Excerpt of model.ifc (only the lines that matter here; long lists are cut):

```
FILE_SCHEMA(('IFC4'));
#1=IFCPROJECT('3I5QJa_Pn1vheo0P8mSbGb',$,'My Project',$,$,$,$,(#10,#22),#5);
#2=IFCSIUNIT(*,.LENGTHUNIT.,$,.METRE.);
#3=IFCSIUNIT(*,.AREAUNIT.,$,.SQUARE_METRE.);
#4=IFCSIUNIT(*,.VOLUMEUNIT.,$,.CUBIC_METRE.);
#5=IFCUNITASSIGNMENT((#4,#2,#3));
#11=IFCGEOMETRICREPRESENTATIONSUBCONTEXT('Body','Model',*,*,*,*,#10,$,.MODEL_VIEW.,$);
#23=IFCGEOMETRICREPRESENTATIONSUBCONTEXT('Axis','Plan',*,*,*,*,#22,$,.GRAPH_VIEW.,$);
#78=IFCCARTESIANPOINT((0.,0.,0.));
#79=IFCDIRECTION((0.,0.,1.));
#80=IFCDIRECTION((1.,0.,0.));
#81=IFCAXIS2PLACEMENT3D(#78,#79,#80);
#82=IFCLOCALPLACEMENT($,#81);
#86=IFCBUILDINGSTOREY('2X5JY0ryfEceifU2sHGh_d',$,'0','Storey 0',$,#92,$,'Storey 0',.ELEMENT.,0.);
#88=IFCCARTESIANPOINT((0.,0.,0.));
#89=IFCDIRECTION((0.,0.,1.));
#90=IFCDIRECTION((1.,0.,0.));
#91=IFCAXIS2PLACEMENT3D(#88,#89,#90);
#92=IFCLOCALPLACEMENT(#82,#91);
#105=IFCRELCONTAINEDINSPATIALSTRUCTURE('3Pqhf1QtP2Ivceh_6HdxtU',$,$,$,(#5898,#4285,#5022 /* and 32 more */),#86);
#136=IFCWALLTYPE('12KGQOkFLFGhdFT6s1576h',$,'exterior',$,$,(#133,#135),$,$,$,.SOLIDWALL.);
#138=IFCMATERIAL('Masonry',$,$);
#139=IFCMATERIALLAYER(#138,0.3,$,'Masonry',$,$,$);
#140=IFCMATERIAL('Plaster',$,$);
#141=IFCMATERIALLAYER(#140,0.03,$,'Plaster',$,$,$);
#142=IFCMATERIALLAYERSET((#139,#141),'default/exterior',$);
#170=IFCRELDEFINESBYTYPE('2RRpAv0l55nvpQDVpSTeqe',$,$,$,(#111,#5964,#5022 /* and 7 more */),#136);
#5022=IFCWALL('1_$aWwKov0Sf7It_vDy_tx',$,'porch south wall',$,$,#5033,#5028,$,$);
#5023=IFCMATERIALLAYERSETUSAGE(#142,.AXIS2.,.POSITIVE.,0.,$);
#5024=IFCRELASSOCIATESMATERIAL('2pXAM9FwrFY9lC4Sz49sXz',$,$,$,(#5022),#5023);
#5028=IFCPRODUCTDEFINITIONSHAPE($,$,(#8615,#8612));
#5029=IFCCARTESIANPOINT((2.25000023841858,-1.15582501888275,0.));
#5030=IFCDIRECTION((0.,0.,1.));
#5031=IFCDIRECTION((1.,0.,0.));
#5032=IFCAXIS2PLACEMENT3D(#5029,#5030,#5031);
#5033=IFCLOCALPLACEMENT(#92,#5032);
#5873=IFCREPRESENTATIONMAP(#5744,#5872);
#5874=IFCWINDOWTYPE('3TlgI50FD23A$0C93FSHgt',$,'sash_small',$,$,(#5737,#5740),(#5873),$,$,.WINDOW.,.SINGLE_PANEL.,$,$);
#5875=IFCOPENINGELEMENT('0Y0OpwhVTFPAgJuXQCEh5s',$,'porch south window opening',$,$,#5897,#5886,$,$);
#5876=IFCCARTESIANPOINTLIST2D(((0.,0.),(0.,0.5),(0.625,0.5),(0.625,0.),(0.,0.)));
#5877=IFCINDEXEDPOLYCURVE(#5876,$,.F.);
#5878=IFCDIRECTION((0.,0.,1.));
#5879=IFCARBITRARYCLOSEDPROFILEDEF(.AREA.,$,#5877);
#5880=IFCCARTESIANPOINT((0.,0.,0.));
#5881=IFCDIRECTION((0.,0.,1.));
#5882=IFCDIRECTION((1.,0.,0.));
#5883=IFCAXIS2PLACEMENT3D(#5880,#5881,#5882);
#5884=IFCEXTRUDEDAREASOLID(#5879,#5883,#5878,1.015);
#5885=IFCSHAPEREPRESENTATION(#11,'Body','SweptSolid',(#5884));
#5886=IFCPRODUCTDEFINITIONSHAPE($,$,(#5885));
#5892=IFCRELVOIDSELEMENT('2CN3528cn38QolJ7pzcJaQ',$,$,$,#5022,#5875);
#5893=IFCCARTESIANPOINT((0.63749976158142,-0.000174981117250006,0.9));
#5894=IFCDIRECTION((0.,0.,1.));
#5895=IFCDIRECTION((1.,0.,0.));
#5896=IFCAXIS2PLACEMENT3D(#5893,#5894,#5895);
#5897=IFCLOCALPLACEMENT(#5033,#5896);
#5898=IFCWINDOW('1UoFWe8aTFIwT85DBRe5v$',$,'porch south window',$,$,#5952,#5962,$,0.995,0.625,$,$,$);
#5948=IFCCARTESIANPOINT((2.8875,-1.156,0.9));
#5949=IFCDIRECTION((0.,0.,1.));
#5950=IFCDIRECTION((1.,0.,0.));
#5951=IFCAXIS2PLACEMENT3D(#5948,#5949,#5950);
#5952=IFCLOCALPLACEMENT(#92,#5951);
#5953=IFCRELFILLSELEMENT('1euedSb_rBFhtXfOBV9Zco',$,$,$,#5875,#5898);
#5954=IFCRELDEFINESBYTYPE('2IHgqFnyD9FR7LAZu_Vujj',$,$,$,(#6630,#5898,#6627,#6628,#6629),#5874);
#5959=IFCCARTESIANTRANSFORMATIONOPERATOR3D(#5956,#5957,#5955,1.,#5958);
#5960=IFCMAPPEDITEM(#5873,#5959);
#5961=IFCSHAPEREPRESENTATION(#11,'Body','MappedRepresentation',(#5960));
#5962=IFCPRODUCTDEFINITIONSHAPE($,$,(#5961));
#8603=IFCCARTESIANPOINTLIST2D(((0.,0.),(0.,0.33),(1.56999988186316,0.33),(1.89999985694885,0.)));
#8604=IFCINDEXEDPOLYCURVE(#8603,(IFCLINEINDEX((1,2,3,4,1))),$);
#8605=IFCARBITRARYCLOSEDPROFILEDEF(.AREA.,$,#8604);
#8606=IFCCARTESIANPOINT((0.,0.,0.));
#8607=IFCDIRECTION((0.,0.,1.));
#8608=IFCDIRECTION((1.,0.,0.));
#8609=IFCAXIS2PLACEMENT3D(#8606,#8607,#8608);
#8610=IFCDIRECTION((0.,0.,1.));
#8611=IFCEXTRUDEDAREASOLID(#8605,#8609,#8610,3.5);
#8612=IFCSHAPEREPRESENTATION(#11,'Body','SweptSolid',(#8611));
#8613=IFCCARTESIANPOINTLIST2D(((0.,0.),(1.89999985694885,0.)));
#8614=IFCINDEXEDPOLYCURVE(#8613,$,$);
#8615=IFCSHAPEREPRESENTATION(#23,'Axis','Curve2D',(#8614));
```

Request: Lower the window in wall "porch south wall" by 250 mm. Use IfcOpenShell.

```python
import numpy as np
import ifcopenshell
import ifcopenshell.api.geometry
import ifcopenshell.util.placement
import ifcopenshell.util.unit

model = ifcopenshell.open("model.ifc")
unit_scale = ifcopenshell.util.unit.calculate_unit_scale(model)

window = model.by_guid("1UoFWe8aTFIwT85DBRe5v$")
opening = window.FillsVoids[0].RelatingOpeningElement
dz = -0.25

shift = np.array([0.0, 0.0, dz])
# The window is not placed relative to its opening, so move both.
for product in (opening, window):
    matrix = ifcopenshell.util.placement.get_local_placement(product.ObjectPlacement)
    matrix[:3, 3] += shift
    ifcopenshell.api.geometry.edit_object_placement(model, product=product, matrix=matrix, is_si=False)

print(f"moved by {dz * unit_scale:+.3f} m")

model.write("model_v2.ifc")
```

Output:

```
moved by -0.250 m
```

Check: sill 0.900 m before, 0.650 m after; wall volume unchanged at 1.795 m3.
